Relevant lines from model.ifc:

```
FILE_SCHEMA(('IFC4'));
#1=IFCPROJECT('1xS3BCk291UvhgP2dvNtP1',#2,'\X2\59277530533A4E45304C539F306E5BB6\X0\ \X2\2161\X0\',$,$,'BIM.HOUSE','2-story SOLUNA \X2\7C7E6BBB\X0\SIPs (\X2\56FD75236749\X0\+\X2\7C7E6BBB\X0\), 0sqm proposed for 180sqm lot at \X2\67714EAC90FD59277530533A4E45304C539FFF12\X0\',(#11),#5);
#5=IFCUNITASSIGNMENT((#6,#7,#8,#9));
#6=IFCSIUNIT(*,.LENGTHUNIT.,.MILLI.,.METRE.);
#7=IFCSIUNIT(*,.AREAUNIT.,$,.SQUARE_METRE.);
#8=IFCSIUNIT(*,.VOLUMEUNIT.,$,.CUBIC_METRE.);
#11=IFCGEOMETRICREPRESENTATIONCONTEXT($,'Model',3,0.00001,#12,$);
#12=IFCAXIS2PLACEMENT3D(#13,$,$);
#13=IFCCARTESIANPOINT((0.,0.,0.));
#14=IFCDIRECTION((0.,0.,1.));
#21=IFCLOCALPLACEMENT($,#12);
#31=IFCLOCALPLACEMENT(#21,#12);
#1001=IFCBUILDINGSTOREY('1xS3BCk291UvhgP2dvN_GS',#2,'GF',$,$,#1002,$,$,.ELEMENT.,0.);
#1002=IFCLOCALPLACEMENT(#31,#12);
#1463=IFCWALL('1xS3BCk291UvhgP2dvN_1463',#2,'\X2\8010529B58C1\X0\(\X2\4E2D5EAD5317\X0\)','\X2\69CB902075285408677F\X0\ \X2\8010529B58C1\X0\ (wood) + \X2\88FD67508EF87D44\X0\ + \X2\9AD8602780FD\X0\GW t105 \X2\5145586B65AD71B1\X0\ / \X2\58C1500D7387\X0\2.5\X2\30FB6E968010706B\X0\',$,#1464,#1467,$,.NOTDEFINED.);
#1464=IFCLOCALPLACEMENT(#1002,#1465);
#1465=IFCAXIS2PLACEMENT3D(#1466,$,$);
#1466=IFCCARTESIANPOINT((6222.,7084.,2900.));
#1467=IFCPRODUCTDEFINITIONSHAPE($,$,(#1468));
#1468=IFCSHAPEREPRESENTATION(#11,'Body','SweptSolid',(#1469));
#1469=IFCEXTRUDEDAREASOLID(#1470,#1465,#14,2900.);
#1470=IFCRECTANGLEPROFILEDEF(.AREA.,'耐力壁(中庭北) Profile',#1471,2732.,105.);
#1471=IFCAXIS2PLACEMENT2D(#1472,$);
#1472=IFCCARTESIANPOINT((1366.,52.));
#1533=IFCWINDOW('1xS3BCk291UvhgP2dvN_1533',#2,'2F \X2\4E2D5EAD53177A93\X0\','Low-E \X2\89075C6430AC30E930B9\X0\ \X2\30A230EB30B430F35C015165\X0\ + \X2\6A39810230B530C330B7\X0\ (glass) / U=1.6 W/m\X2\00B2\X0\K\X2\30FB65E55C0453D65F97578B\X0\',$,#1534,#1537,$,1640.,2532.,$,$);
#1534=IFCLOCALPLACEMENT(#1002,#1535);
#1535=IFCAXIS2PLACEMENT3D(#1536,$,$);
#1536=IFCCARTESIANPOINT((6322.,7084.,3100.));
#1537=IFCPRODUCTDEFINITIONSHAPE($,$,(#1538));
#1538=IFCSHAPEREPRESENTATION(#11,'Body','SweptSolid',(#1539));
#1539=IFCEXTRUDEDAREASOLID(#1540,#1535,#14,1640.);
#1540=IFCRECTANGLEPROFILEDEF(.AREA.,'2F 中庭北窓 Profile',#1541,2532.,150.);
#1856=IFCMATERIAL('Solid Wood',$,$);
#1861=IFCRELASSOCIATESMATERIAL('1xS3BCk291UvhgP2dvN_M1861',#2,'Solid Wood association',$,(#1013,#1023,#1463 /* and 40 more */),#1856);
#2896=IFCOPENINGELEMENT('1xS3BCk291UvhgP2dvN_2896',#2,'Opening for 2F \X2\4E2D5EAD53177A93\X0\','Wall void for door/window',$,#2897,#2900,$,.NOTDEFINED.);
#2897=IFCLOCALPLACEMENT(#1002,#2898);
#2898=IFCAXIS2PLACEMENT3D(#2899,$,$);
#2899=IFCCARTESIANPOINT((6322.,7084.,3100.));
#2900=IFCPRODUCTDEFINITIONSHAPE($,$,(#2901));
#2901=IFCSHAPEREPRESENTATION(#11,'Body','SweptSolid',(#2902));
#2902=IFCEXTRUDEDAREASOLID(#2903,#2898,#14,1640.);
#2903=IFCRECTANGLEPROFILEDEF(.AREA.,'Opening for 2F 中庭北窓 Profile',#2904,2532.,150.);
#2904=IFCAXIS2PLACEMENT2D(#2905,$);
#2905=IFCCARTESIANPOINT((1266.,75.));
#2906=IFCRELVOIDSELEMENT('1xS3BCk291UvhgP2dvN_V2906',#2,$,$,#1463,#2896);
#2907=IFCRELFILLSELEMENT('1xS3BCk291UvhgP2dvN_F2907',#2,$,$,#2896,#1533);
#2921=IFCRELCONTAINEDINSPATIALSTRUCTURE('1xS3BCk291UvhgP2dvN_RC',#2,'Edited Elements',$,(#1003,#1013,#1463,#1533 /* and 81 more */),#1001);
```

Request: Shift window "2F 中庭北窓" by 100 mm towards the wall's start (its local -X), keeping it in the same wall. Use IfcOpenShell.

```python
import ifcopenshell
import ifcopenshell.api.geometry
import ifcopenshell.util.placement
import ifcopenshell.util.unit

model = ifcopenshell.open("model.ifc")
unit_scale = ifcopenshell.util.unit.calculate_unit_scale(model)

window = model.by_guid("1xS3BCk291UvhgP2dvN_1533")
opening = window.FillsVoids[0].RelatingOpeningElement
wall = opening.VoidsElements[0].RelatingBuildingElement

wall_matrix = ifcopenshell.util.placement.get_local_placement(wall.ObjectPlacement)
shift = wall_matrix[:3, 0] * -0.1 / unit_scale
before = ifcopenshell.util.placement.get_local_placement(window.ObjectPlacement)[:3, 3].copy()

# The window is not placed relative to its opening, so move both.
for product in (opening, window):
    matrix = ifcopenshell.util.placement.get_local_placement(product.ObjectPlacement)
    matrix[:3, 3] += shift
    ifcopenshell.api.geometry.edit_object_placement(model, product=product, matrix=matrix, is_si=False)

after = ifcopenshell.util.placement.get_local_placement(window.ObjectPlacement)[:3, 3]
print("window moved by", (after - before).round(3) + 0.0)

model.write("model-out.ifc")
```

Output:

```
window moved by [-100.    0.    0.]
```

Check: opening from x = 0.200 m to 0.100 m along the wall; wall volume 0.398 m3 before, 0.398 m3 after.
